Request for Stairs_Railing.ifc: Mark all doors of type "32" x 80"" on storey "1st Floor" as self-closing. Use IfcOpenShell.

First a look at what the model holds.

```python
import ifcopenshell
import ifcopenshell.util.element

model = ifcopenshell.open("Stairs_Railing.ifc")
print(model.schema)
storey = next(s for s in model.by_type("IfcBuildingStorey") if s.Name == "1st Floor")
doors = [e for e in ifcopenshell.util.element.get_decomposition(storey) if e.is_a("IfcDoor")]
seen = {}
for e in doors:
    element_type = ifcopenshell.util.element.get_type(e)
    key = (element_type.Name if element_type != e and element_type else None, ifcopenshell.util.element.get_pset(e, "Pset_DoorCommon", "SelfClosing"))
    seen[key] = seen.get(key, 0) + 1
for (name, value), count in sorted(seen.items(), key=str):
    print(count, "x", name, "|", value)
```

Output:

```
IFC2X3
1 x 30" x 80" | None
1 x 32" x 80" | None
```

```python
import ifcopenshell
import ifcopenshell.api.pset
import ifcopenshell.util.element

model = ifcopenshell.open("Stairs_Railing.ifc")

storey = next(s for s in model.by_type("IfcBuildingStorey") if s.Name == "1st Floor")
doors = [e for e in ifcopenshell.util.element.get_decomposition(storey) if e.is_a("IfcDoor")]

count = 0
for e in doors:
    element_type = ifcopenshell.util.element.get_type(e)
    if element_type in (None, e) or element_type.Name != '32" x 80"':
        continue
    # add_pset returns the element's existing set when there is one.
    pset = ifcopenshell.api.pset.add_pset(model, product=e, name="Pset_DoorCommon")
    ifcopenshell.api.pset.edit_pset(model, pset=pset, properties={"SelfClosing": True})
    count += 1

print(count, "doors updated")

model.write("Stairs_Railing_v2.ifc")
```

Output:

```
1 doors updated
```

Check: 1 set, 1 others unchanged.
